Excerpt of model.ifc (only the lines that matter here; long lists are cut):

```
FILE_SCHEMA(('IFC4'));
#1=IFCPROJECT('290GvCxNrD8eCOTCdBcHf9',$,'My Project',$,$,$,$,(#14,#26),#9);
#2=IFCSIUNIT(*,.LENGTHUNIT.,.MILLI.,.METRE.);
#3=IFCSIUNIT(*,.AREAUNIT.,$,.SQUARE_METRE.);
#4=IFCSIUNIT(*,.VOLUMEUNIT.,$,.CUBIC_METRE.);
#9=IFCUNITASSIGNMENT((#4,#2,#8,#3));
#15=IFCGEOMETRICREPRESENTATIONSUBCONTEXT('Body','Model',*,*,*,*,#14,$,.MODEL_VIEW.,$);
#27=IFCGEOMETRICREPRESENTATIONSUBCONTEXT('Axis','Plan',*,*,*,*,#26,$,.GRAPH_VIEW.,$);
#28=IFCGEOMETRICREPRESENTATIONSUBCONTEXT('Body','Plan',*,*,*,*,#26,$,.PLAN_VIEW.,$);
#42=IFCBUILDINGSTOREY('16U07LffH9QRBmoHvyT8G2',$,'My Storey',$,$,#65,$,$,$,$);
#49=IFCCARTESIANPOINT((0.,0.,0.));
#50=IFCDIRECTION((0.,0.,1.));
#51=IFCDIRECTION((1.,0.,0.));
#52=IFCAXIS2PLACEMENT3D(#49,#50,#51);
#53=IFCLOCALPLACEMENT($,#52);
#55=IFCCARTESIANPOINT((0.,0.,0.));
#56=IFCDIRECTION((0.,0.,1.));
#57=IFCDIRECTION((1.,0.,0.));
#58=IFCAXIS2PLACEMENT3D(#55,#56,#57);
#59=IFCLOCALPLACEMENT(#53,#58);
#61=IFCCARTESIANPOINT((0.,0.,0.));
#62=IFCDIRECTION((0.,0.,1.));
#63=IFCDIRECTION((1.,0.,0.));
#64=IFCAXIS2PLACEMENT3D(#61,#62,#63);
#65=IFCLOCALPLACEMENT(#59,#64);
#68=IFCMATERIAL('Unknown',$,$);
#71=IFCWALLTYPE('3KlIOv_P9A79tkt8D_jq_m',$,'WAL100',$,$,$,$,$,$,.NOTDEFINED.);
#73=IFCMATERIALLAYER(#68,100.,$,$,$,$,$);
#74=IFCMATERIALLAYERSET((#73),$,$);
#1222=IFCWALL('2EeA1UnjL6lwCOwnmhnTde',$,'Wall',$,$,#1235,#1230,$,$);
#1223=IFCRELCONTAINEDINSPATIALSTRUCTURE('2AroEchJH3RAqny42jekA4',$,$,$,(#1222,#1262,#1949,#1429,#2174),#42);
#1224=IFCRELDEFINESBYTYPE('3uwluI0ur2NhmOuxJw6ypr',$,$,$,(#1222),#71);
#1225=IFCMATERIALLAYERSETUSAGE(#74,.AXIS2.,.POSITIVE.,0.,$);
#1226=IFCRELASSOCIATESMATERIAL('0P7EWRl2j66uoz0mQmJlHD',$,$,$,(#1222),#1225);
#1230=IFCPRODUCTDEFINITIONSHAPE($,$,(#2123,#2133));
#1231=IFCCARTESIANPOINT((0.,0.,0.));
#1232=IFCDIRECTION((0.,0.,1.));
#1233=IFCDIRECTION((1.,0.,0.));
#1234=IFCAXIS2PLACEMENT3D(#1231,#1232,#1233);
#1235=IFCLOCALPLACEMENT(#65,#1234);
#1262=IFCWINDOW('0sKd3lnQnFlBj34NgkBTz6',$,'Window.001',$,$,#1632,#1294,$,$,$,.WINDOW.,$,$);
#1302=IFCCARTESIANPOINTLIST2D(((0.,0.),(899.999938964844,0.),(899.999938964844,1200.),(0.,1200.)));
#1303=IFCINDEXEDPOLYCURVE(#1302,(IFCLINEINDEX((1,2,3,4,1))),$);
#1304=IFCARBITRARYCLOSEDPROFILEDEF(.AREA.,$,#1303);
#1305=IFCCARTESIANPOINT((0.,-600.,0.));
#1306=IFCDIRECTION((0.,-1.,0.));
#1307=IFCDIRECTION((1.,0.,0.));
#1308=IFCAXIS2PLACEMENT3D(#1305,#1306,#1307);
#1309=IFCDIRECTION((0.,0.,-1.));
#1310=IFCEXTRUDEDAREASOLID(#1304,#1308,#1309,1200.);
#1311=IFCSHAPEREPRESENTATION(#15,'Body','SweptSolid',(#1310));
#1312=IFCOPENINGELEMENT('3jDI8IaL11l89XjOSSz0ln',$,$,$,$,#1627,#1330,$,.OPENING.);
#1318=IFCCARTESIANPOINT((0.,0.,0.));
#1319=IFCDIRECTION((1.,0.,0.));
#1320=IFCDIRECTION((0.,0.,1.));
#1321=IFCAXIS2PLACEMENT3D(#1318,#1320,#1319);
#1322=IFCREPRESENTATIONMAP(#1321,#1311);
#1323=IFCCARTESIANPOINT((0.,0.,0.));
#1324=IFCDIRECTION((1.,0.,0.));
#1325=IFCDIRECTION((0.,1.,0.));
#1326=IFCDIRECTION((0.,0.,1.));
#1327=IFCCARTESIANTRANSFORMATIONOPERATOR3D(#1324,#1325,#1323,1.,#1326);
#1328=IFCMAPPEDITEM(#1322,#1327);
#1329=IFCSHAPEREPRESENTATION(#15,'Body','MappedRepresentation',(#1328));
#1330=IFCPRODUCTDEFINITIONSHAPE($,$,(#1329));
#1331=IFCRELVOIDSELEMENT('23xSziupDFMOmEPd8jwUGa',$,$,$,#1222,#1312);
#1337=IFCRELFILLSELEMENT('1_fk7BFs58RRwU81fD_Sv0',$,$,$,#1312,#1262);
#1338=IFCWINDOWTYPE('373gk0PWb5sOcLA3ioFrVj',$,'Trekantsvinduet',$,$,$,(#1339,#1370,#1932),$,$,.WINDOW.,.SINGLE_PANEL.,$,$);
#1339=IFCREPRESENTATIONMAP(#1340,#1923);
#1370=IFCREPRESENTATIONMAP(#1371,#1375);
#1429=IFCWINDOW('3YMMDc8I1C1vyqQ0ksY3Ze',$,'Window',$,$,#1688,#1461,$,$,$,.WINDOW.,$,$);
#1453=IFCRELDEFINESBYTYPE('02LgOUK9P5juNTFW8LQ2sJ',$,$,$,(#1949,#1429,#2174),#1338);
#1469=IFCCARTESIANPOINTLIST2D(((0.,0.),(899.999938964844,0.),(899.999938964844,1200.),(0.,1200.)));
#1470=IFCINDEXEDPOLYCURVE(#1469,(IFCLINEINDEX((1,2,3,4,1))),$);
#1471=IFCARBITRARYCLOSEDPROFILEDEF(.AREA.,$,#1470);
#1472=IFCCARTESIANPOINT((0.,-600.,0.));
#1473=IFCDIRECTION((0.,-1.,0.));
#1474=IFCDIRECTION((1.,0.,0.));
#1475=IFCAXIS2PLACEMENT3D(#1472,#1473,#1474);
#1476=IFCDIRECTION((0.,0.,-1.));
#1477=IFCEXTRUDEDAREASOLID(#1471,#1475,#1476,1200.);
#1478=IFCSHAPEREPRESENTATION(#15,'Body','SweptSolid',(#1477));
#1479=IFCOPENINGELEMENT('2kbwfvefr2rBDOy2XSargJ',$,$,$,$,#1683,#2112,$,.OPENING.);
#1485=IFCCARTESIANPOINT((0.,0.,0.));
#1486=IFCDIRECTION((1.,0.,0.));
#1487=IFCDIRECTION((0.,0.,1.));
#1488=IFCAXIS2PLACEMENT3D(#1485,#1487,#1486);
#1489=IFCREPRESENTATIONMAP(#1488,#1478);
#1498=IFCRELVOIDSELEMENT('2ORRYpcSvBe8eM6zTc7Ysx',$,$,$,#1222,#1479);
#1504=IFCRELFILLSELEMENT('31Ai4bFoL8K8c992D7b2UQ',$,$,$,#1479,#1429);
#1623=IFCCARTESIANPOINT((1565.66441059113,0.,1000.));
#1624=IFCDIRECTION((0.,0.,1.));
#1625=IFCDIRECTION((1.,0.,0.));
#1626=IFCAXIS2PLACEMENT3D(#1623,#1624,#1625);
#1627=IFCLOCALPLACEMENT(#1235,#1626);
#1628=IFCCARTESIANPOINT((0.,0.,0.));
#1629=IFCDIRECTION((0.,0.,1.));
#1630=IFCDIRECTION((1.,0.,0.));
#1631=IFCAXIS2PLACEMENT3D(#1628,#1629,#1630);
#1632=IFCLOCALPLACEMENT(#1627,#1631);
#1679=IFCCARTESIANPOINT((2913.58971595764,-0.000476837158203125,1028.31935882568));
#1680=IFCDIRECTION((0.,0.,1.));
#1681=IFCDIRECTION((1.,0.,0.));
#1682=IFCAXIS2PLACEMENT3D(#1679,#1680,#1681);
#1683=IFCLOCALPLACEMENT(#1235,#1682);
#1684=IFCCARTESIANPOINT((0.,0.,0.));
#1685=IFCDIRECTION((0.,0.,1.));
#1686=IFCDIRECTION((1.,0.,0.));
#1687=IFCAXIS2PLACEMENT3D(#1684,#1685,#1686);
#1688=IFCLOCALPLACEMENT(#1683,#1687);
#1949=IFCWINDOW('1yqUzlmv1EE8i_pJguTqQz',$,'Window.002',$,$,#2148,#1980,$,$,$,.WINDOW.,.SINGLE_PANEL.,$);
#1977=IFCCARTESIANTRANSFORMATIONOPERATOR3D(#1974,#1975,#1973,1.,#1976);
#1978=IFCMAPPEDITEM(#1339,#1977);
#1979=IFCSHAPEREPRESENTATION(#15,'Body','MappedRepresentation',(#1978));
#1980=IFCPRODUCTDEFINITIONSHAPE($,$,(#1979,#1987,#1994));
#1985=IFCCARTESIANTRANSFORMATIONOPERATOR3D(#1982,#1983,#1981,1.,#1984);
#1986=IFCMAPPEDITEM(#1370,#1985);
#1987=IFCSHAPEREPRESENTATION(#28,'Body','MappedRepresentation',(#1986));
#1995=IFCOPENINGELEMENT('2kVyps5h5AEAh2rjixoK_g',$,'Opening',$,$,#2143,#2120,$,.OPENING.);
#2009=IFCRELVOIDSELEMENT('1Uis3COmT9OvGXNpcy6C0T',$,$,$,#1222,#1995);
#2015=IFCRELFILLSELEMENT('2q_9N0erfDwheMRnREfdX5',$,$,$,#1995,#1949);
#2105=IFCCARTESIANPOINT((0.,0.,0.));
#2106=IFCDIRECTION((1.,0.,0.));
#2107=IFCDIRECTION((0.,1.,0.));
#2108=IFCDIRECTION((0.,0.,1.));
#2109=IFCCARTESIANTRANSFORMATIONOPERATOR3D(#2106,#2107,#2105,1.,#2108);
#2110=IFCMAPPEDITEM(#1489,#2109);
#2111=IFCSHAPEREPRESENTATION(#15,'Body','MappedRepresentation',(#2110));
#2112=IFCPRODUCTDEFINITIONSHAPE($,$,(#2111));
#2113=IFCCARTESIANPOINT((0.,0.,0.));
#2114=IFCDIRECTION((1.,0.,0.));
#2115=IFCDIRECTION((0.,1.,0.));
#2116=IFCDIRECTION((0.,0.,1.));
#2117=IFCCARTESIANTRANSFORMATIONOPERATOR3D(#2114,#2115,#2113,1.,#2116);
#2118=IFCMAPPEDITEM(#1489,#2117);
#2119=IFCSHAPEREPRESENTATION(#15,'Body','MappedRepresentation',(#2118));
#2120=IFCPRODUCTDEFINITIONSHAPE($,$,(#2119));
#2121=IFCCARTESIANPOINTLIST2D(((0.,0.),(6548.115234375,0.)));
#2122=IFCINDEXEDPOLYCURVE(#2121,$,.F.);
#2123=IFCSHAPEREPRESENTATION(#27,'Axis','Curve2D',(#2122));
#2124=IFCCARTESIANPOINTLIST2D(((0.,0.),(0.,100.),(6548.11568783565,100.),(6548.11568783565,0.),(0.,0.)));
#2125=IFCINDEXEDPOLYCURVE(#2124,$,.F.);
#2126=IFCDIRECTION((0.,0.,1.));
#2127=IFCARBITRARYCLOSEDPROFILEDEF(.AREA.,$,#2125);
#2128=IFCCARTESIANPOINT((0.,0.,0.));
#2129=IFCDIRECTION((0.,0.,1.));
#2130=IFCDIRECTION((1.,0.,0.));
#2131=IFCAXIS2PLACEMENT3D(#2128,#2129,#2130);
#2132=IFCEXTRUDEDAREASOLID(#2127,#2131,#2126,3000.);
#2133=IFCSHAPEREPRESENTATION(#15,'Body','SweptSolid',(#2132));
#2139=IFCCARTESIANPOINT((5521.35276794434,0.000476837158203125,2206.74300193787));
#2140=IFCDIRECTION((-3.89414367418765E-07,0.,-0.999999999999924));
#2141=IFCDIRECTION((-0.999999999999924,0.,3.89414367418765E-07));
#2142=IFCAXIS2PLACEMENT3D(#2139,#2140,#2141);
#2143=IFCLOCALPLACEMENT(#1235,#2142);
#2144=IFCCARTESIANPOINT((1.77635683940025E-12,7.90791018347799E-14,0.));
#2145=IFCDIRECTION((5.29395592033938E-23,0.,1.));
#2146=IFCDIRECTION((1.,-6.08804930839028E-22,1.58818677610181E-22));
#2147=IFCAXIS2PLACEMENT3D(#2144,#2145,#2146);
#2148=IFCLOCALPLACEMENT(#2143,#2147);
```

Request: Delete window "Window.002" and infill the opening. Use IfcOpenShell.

```python
import ifcopenshell
import ifcopenshell.api.feature
import ifcopenshell.api.root
import ifcopenshell.geom
import ifcopenshell.util.shape

model = ifcopenshell.open("model.ifc")
settings = ifcopenshell.geom.settings()


def volume(element):
    """Net volume in cubic metres, openings subtracted."""
    shape = ifcopenshell.geom.create_shape(settings, element)
    return ifcopenshell.util.shape.get_volume(shape.geometry)


window = model.by_id(1949)
opening = window.FillsVoids[0].RelatingOpeningElement
wall = opening.VoidsElements[0].RelatingBuildingElement
before = volume(wall)

ifcopenshell.api.root.remove_product(model, product=window)
ifcopenshell.api.feature.remove_feature(model, feature=opening)

after = volume(wall)

print(f"wall volume {before:.3f} -> {after:.3f} m3")

model.write("model-out.ifc")
```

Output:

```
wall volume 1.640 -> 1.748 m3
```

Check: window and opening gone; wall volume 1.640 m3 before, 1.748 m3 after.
